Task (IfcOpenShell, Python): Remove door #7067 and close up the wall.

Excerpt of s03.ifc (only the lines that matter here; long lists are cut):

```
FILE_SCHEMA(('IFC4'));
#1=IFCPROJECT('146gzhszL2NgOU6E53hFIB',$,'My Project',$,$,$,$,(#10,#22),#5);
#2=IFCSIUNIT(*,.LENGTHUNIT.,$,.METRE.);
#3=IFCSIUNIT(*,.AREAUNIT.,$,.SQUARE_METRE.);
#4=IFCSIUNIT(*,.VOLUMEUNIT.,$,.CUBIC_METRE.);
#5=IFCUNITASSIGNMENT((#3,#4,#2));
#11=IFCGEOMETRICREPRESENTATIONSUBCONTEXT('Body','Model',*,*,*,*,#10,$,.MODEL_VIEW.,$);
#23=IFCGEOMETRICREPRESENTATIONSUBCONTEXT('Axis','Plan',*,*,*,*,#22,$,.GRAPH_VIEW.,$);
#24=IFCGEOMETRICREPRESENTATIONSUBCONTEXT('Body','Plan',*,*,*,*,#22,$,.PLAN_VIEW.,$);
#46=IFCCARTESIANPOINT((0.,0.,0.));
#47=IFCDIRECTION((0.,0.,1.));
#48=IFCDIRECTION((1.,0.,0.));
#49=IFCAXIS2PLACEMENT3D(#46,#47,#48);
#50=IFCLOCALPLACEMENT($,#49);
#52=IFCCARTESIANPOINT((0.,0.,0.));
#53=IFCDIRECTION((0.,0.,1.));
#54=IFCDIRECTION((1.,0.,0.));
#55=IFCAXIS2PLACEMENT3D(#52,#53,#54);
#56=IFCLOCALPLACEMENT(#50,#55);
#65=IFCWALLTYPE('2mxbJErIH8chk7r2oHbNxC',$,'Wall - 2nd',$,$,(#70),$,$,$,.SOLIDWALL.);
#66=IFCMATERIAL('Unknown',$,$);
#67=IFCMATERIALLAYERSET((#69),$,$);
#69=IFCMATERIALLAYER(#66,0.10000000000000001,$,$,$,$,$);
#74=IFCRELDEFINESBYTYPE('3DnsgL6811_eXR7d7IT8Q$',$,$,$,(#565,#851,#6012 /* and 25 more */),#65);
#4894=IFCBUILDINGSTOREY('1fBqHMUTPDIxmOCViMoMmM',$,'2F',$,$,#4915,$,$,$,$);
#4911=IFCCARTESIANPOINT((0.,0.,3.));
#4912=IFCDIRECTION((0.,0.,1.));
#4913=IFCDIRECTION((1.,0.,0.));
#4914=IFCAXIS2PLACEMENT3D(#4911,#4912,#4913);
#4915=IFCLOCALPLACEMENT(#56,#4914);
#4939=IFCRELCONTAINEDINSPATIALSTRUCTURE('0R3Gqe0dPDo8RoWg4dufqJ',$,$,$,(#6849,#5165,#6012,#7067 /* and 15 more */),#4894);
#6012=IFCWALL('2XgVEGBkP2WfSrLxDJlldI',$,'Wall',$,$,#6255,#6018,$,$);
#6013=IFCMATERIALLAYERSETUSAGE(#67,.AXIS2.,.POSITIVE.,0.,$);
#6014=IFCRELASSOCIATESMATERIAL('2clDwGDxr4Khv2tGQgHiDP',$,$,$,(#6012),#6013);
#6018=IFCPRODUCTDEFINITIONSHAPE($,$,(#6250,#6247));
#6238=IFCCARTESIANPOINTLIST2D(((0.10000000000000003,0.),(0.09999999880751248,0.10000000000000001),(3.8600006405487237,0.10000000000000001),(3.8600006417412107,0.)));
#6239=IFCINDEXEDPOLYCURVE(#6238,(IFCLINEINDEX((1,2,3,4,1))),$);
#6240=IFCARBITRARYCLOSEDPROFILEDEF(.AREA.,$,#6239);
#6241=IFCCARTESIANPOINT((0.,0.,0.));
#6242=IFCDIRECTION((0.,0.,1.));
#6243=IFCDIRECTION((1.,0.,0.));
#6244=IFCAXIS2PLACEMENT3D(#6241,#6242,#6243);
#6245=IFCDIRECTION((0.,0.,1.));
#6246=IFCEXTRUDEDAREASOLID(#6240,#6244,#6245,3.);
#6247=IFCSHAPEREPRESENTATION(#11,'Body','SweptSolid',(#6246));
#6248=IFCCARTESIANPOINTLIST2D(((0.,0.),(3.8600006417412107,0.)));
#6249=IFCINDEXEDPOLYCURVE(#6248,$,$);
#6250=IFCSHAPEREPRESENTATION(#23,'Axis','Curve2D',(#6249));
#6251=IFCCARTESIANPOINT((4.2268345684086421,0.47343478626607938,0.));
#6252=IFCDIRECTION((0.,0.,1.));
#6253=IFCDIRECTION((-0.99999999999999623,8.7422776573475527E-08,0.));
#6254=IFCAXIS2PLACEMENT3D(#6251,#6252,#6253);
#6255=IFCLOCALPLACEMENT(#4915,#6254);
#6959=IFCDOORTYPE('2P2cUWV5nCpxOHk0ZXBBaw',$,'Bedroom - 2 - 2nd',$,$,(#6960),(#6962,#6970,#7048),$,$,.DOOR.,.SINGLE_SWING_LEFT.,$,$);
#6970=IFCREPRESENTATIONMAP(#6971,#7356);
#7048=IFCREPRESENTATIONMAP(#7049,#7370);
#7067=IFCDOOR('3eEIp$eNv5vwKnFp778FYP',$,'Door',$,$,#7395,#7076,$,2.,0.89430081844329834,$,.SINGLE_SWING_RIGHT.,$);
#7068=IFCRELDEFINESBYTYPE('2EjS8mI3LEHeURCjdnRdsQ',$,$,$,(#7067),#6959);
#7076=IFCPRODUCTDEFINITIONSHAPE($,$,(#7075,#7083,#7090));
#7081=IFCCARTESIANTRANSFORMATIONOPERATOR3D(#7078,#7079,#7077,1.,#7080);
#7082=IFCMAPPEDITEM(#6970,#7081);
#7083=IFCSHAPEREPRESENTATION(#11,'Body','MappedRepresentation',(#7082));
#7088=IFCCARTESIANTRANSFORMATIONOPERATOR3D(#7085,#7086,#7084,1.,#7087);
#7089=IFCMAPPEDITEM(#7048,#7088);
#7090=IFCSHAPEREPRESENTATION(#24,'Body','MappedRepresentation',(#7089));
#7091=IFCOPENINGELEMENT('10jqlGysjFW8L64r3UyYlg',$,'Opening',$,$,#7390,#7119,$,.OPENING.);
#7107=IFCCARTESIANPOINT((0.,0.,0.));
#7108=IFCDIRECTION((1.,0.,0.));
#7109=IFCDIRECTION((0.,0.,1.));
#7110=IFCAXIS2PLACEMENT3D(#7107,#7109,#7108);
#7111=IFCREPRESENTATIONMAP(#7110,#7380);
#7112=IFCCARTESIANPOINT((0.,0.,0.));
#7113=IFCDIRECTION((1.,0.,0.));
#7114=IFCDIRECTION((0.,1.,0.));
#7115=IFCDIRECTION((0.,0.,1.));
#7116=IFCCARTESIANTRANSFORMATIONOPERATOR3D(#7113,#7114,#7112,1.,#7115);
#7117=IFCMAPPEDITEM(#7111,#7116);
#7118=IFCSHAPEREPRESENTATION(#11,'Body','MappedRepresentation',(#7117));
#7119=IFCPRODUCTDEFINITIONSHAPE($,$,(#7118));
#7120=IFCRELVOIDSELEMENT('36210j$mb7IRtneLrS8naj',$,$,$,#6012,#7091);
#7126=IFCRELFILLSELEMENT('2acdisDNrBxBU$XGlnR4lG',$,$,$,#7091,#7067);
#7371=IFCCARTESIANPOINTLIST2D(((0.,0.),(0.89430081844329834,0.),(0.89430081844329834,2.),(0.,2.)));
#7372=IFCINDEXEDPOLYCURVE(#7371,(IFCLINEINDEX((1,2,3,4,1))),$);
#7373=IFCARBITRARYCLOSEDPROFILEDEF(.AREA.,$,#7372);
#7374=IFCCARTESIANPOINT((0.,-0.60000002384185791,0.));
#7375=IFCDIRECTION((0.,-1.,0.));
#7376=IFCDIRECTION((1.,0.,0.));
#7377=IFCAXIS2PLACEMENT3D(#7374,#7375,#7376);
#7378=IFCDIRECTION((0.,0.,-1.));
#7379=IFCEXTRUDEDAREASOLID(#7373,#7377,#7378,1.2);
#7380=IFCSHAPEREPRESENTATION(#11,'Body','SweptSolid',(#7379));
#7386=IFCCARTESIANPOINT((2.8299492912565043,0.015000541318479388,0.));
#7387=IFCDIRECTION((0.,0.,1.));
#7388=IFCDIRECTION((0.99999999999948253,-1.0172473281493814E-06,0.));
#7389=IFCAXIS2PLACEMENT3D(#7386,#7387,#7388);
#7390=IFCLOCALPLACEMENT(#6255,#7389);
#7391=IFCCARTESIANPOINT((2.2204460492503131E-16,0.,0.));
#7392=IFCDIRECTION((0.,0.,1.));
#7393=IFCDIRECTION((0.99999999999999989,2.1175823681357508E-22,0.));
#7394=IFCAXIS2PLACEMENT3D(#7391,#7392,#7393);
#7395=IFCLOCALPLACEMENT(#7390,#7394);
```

```python
import ifcopenshell
import ifcopenshell.api.feature
import ifcopenshell.api.root
import ifcopenshell.geom
import ifcopenshell.util.shape

model = ifcopenshell.open("s03.ifc")
settings = ifcopenshell.geom.settings()


def volume(element):
    """Net volume in cubic metres, openings subtracted."""
    shape = ifcopenshell.geom.create_shape(settings, element)
    return ifcopenshell.util.shape.get_volume(shape.geometry)


door = model.by_guid("3eEIp$eNv5vwKnFp778FYP")
opening = door.FillsVoids[0].RelatingOpeningElement
wall = opening.VoidsElements[0].RelatingBuildingElement
before = volume(wall)

ifcopenshell.api.root.remove_product(model, product=door)
ifcopenshell.api.feature.remove_feature(model, feature=opening)

after = volume(wall)

print(f"wall volume {before:.3f} -> {after:.3f} m3")

model.write("s03-out.ifc")
```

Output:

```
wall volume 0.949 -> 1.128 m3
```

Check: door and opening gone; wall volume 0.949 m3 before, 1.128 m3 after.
